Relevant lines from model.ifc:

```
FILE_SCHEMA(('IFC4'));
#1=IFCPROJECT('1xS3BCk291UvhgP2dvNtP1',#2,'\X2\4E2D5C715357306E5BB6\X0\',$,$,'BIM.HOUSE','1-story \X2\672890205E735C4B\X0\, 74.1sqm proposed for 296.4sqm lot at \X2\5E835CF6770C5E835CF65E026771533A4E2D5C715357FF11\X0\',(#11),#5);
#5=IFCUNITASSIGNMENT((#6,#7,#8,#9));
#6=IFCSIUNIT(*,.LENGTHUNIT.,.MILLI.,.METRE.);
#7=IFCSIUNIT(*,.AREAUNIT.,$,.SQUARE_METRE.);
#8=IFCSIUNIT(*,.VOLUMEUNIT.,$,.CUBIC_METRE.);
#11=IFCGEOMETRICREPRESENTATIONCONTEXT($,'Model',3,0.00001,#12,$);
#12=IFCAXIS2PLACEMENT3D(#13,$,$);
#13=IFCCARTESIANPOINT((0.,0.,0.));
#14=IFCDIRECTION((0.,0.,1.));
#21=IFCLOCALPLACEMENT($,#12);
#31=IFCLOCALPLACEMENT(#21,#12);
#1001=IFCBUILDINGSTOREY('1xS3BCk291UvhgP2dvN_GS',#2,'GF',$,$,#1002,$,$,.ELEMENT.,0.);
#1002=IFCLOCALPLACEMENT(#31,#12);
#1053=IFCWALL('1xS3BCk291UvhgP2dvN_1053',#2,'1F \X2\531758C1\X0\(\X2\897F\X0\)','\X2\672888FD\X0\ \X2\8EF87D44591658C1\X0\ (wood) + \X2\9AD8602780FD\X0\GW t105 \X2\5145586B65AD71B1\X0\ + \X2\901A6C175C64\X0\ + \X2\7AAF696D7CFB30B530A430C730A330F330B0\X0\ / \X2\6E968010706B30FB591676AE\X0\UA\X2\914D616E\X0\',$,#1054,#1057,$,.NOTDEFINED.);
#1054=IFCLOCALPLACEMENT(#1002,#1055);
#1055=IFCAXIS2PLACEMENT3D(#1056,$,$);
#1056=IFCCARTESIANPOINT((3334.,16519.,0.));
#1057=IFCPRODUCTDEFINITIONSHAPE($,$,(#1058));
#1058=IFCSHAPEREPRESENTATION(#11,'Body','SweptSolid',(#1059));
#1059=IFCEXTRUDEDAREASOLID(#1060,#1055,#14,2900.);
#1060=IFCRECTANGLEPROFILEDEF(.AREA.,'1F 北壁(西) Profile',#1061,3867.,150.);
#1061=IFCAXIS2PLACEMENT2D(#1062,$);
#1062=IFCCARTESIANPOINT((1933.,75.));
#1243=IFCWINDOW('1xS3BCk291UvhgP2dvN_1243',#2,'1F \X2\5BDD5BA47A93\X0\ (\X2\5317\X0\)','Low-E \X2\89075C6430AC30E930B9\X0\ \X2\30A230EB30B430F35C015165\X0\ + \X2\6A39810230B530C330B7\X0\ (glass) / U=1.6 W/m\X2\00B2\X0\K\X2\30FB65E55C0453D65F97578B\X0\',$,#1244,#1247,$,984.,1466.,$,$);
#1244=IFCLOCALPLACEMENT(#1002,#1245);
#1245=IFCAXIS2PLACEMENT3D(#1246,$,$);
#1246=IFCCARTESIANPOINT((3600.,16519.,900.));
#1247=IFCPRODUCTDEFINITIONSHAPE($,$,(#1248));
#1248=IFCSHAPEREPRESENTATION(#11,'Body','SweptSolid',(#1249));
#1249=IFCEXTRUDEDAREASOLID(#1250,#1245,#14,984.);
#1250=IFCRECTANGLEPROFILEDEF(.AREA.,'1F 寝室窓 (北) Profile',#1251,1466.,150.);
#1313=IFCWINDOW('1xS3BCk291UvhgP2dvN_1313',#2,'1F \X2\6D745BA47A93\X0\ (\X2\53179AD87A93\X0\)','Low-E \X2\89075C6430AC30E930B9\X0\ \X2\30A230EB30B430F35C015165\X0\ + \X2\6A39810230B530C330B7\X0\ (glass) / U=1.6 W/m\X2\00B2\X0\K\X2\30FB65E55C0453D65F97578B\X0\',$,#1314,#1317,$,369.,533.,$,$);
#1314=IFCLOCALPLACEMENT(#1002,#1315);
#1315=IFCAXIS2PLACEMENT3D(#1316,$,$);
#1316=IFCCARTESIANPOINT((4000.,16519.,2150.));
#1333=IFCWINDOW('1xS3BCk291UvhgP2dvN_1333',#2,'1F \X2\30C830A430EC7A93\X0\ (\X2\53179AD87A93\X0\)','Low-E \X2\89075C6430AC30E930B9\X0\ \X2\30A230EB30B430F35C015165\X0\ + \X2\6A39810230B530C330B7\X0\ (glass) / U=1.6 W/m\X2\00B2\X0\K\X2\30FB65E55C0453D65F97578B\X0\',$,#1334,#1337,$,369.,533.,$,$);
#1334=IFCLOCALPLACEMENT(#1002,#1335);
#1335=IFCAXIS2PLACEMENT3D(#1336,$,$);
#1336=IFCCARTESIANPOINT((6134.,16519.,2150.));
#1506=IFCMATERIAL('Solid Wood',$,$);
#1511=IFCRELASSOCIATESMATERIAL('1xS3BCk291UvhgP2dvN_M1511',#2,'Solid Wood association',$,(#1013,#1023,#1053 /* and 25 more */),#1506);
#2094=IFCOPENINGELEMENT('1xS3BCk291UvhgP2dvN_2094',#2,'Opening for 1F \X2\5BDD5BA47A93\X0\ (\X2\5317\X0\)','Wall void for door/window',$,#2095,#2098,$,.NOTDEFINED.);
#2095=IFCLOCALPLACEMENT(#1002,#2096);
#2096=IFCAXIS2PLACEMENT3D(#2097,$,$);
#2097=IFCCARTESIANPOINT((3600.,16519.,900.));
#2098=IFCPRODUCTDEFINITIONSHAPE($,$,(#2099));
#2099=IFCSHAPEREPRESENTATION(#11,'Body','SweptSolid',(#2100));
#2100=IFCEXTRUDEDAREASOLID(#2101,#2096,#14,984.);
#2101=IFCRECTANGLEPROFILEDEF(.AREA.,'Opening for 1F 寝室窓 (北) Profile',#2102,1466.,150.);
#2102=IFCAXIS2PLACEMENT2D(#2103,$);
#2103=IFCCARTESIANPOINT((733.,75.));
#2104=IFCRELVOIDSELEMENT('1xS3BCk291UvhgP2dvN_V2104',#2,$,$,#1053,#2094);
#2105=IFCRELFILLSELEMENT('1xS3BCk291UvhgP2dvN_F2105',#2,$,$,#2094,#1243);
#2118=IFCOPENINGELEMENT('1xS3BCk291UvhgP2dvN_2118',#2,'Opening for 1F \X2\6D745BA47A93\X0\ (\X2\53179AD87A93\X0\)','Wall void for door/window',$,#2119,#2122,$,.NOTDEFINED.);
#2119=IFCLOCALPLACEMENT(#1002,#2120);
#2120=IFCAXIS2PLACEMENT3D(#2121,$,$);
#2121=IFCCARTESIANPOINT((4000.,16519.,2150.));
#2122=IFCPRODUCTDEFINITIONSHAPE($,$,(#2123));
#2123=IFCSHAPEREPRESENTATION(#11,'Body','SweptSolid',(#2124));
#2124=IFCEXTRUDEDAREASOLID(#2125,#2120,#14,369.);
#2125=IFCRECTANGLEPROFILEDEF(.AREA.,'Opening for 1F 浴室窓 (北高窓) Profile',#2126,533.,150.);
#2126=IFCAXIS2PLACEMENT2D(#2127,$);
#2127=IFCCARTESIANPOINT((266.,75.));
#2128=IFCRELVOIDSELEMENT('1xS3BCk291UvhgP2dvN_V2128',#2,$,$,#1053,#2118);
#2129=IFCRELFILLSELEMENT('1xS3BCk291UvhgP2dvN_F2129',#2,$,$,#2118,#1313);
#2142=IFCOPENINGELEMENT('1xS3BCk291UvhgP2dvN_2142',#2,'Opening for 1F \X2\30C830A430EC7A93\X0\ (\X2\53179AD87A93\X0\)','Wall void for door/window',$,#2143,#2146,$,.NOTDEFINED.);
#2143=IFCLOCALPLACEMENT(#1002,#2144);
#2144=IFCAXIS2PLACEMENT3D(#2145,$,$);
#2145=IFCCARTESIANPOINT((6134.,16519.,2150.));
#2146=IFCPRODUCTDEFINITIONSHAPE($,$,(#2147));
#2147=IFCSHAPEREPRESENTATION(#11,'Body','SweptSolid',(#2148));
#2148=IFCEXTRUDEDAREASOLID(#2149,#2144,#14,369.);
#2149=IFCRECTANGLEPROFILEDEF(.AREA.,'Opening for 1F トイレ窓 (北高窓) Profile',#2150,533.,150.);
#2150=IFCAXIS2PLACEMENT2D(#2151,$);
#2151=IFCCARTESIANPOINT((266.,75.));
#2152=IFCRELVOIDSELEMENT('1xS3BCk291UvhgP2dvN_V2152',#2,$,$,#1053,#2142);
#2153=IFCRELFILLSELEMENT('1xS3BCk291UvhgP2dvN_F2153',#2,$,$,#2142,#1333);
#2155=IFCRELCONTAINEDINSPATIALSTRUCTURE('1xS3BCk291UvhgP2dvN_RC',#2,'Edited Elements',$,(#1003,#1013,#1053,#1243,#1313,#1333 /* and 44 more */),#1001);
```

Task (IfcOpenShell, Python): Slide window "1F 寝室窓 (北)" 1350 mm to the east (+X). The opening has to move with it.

```python
import ifcopenshell
import ifcopenshell.api.geometry
import ifcopenshell.util.placement

model = ifcopenshell.open("model.ifc")

window = model.by_id(1243)
opening = window.FillsVoids[0].RelatingOpeningElement
wall = opening.VoidsElements[0].RelatingBuildingElement

wall_matrix = ifcopenshell.util.placement.get_local_placement(wall.ObjectPlacement)
shift = wall_matrix[:3, 0] * 1350.0
before = ifcopenshell.util.placement.get_local_placement(window.ObjectPlacement)[:3, 3].copy()

# The window is not placed relative to its opening, so move both.
for product in (opening, window):
    matrix = ifcopenshell.util.placement.get_local_placement(product.ObjectPlacement)
    matrix[:3, 3] += shift
    ifcopenshell.api.geometry.edit_object_placement(model, product=product, matrix=matrix, is_si=False)

after = ifcopenshell.util.placement.get_local_placement(window.ObjectPlacement)[:3, 3]
print("window moved by", (after - before).round(3) + 0.0)

model.write("model_rev.ifc")
```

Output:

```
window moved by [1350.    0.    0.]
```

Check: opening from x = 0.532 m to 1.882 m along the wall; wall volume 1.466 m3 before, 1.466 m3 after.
